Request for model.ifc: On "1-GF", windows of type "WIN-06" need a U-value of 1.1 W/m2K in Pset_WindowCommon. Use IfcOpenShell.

First a look at what the model holds.

```python
import ifcopenshell
import ifcopenshell.util.element

model = ifcopenshell.open("model.ifc")
print(model.schema)
storey = next(s for s in model.by_type("IfcBuildingStorey") if s.Name == "1-GF")
windows = [e for e in ifcopenshell.util.element.get_decomposition(storey) if e.is_a("IfcWindow")]
seen = {}
for e in windows:
    element_type = ifcopenshell.util.element.get_type(e)
    key = (element_type.Name if element_type != e and element_type else None, ifcopenshell.util.element.get_pset(e, "Pset_WindowCommon", "ThermalTransmittance"))
    seen[key] = seen.get(key, 0) + 1
for (name, value), count in sorted(seen.items(), key=str):
    print(count, "x", name, "|", value)
```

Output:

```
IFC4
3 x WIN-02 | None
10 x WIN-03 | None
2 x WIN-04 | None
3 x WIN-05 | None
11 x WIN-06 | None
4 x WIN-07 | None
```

```python
import ifcopenshell
import ifcopenshell.api.pset
import ifcopenshell.util.element

model = ifcopenshell.open("model.ifc")

storey = next(s for s in model.by_type("IfcBuildingStorey") if s.Name == "1-GF")
windows = [e for e in ifcopenshell.util.element.get_decomposition(storey) if e.is_a("IfcWindow")]

count = 0
for e in windows:
    element_type = ifcopenshell.util.element.get_type(e)
    if element_type in (None, e) or element_type.Name != "WIN-06":
        continue
    # add_pset returns the element's existing set when there is one.
    pset = ifcopenshell.api.pset.add_pset(model, product=e, name="Pset_WindowCommon")
    ifcopenshell.api.pset.edit_pset(model, pset=pset, properties={"ThermalTransmittance": 1.1})
    count += 1

print(count, "windows updated")

model.write("model_updated.ifc")
```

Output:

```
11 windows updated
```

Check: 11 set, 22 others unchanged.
